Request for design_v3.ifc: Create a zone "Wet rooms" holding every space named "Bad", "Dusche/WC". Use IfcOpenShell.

First a look at what the model holds.

```python
import ifcopenshell

model = ifcopenshell.open("design_v3.ifc")
print(model.schema)
seen = {}
for space in model.by_type("IfcSpace"):
    seen[space.LongName] = seen.get(space.LongName, 0) + 1
for name, count in sorted(seen.items(), key=str):
    print(count, "x", name)
print("zones:", [z.Name for z in model.by_type("IfcZone")][:20])
```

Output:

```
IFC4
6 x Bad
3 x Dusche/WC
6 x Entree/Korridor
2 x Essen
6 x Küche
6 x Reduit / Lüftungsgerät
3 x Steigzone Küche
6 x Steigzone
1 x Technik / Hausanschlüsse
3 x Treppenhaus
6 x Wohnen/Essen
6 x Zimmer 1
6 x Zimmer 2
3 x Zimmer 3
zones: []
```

```python
import ifcopenshell
import ifcopenshell.api.group
import ifcopenshell.api.root

model = ifcopenshell.open("design_v3.ifc")

names = {"Bad", "Dusche/WC"}
spaces = [s for s in model.by_type("IfcSpace") if s.LongName in names]

zone = ifcopenshell.api.root.create_entity(model, ifc_class="IfcZone", name="Wet rooms")
ifcopenshell.api.group.assign_group(model, products=spaces, group=zone)
print(len(spaces), "spaces in", zone.Name)

model.write("design_v3_rev.ifc")
```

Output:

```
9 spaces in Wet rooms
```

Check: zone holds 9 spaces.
